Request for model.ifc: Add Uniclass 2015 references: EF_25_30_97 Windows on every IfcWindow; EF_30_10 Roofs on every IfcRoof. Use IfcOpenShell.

First a look at what the model holds.

```python
import ifcopenshell

model = ifcopenshell.open("model.ifc")
print(model.schema)
print("classifications:", [c.Name for c in model.by_type("IfcClassification")])
for ifc_class in ("IfcDoor", "IfcRoof", "IfcStair", "IfcWall", "IfcWindow"):
    print(ifc_class, len(model.by_type(ifc_class)))
```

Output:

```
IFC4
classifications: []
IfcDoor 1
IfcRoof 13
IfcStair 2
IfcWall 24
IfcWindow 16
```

```python
import ifcopenshell
import ifcopenshell.api.classification

model = ifcopenshell.open("model.ifc")

system = ifcopenshell.api.classification.add_classification(model, classification="Uniclass 2015")

codes = {
    "IfcWindow": ("EF_25_30_97", "Windows"),
    "IfcRoof": ("EF_30_10", "Roofs"),
}
for ifc_class, (code, name) in codes.items():
    products = model.by_type(ifc_class)
    ifcopenshell.api.classification.add_reference(
        model, products=products, classification=system, identification=code, name=name
    )
    print(code, len(products))

model.write("model-out.ifc")
```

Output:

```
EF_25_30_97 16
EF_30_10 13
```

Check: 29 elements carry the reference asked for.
